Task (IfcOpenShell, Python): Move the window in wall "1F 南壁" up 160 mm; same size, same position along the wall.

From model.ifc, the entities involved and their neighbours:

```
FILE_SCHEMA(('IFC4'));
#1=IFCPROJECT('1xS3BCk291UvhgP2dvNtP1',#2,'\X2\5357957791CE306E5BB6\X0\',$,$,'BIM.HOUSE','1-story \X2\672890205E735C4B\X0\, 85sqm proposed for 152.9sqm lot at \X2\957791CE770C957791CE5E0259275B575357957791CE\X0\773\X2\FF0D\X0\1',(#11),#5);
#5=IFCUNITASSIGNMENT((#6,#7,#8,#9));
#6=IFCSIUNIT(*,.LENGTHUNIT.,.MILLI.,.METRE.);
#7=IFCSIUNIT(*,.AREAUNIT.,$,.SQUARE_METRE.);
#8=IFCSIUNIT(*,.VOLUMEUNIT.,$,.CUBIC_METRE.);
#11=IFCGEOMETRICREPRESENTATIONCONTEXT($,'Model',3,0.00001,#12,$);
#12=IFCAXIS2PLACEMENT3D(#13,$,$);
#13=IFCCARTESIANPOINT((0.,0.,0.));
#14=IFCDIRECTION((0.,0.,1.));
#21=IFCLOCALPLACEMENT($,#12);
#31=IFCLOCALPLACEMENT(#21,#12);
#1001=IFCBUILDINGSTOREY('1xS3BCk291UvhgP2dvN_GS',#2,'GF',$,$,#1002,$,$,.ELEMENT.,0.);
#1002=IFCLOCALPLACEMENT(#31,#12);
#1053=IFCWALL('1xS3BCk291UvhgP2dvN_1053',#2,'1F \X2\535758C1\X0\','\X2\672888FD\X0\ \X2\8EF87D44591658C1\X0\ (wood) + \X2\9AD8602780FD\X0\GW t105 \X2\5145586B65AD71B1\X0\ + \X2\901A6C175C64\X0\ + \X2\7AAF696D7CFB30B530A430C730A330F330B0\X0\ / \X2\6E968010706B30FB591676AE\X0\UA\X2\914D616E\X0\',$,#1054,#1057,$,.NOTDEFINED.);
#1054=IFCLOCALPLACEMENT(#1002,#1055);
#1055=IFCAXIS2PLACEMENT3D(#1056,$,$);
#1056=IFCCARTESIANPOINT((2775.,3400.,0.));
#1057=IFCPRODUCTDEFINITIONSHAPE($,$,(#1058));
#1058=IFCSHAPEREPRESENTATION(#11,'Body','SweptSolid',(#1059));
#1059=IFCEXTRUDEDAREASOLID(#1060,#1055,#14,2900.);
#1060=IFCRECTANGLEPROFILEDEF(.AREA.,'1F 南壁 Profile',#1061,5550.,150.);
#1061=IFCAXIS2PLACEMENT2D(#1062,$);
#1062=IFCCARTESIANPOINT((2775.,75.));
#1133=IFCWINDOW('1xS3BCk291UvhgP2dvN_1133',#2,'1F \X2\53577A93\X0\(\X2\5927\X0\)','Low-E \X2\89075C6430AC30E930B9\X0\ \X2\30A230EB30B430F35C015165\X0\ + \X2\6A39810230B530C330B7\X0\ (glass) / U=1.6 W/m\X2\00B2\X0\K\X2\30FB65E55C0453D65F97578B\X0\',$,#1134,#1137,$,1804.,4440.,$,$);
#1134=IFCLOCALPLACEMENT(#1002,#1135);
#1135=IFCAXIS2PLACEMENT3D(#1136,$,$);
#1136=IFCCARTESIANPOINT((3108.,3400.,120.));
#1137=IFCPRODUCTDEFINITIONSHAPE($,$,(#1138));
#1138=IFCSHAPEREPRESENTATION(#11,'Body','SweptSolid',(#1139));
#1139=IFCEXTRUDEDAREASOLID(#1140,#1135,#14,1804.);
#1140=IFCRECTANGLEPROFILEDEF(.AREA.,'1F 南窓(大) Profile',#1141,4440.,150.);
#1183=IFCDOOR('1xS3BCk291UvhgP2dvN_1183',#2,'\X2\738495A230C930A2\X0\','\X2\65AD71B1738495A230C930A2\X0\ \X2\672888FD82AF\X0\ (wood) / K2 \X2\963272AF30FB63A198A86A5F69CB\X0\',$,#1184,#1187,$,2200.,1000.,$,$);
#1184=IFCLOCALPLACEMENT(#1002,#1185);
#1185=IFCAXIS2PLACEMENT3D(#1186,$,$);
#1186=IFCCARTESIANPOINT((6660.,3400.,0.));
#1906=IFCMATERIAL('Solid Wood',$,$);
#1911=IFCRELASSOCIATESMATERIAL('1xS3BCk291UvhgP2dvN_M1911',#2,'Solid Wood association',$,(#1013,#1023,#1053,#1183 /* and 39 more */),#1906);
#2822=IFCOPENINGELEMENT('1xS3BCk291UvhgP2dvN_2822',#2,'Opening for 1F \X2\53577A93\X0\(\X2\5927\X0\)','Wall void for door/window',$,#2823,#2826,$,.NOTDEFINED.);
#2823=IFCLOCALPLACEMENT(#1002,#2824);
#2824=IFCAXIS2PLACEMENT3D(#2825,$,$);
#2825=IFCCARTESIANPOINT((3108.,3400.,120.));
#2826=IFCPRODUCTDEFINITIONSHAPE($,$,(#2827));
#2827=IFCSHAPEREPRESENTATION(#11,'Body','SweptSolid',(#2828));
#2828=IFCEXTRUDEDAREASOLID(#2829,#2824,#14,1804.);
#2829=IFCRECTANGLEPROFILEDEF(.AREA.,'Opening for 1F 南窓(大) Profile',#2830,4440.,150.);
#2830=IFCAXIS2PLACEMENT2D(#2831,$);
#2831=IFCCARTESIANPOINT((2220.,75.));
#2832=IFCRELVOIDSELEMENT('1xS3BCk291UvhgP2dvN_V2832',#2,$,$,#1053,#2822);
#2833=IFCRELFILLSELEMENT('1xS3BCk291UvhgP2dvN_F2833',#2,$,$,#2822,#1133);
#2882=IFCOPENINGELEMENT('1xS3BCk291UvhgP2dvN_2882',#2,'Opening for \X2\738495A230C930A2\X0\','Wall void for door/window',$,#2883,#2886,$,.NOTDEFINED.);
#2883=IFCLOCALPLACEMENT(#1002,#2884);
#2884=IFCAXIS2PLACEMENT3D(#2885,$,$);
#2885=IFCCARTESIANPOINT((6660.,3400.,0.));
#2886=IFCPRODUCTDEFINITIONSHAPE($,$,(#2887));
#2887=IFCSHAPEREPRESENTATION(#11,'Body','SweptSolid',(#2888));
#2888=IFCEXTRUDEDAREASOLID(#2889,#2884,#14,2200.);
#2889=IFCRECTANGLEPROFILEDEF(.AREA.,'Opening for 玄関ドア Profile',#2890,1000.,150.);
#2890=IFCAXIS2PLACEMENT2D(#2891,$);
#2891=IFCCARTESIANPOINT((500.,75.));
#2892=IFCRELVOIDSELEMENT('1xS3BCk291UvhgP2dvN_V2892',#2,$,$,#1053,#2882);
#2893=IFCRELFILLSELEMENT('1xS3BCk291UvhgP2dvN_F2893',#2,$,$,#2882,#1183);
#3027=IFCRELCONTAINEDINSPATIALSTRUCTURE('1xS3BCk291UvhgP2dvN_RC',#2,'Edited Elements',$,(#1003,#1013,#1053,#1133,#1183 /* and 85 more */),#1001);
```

```python
import numpy as np
import ifcopenshell
import ifcopenshell.api.geometry
import ifcopenshell.util.placement
import ifcopenshell.util.unit

model = ifcopenshell.open("model.ifc")
unit_scale = ifcopenshell.util.unit.calculate_unit_scale(model)

window = model.by_guid("1xS3BCk291UvhgP2dvN_1133")
opening = window.FillsVoids[0].RelatingOpeningElement
dz = 0.16 / unit_scale

shift = np.array([0.0, 0.0, dz])
# The window is not placed relative to its opening, so move both.
for product in (opening, window):
    matrix = ifcopenshell.util.placement.get_local_placement(product.ObjectPlacement)
    matrix[:3, 3] += shift
    ifcopenshell.api.geometry.edit_object_placement(model, product=product, matrix=matrix, is_si=False)

print(f"moved by {dz * unit_scale:+.3f} m")

model.write("model_v2.ifc")
```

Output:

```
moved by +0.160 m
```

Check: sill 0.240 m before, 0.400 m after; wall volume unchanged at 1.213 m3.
